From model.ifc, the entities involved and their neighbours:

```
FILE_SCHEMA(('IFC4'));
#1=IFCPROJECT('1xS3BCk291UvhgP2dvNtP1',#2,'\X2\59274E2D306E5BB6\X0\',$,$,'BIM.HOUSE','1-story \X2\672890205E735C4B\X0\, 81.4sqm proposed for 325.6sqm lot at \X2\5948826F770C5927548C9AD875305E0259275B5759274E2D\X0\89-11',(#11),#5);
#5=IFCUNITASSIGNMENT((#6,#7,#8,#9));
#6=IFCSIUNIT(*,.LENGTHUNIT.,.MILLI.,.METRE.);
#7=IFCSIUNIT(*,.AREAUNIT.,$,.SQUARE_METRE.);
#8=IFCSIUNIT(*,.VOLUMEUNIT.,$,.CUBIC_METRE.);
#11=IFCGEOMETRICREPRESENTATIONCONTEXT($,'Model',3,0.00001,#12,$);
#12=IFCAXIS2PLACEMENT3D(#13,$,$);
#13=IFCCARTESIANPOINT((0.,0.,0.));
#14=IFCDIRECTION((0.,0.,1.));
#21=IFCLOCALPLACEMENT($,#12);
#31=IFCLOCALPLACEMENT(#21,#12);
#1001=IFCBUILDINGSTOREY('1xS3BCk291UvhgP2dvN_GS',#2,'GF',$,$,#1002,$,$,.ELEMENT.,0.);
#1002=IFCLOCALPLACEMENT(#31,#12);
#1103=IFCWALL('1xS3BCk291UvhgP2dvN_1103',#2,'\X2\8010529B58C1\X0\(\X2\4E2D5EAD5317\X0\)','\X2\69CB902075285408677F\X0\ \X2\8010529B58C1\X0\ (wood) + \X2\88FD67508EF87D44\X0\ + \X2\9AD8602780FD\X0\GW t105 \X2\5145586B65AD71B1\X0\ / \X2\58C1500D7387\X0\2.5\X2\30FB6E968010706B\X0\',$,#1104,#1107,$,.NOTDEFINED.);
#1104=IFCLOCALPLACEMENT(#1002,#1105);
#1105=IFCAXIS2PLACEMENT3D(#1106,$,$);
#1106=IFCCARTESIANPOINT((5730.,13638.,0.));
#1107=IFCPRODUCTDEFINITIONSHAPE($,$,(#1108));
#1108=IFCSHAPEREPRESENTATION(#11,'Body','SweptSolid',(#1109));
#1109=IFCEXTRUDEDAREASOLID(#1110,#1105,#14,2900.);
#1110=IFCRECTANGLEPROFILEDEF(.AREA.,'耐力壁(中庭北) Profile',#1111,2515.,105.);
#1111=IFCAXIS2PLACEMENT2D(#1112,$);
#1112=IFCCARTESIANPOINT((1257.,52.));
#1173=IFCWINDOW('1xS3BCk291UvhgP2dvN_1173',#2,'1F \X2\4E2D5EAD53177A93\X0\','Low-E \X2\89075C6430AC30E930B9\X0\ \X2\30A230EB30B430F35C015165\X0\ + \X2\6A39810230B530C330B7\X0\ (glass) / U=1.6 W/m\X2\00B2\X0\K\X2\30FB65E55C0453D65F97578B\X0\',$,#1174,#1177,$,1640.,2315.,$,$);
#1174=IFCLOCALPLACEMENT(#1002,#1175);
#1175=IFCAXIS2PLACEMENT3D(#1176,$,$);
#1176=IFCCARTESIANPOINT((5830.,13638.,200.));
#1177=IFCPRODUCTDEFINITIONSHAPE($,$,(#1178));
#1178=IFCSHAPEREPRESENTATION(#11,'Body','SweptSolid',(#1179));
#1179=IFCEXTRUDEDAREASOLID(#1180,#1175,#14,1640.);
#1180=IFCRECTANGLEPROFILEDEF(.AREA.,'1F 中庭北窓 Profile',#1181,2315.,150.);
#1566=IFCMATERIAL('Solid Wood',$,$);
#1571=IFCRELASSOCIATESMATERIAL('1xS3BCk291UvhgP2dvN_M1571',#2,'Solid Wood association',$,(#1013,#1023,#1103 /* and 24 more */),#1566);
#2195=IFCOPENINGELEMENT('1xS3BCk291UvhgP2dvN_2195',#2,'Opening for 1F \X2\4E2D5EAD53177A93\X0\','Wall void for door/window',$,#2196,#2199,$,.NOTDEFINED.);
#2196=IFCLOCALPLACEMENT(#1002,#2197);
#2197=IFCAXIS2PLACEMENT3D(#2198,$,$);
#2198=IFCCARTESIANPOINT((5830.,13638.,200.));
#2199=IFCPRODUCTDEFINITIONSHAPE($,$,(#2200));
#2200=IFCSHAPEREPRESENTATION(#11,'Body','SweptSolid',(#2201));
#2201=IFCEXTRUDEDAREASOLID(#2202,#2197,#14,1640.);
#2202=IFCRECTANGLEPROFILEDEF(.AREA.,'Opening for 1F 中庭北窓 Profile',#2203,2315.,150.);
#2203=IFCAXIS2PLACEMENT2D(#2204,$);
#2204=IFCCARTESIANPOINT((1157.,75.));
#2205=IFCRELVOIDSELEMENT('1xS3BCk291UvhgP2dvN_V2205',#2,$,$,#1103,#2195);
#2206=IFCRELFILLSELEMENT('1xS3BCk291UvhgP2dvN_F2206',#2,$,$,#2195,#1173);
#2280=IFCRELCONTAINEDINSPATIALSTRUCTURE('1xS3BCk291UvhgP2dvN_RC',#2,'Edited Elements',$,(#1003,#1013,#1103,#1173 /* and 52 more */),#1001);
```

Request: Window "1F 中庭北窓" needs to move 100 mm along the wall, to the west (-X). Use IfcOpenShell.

```python
import ifcopenshell
import ifcopenshell.api.geometry
import ifcopenshell.util.placement

model = ifcopenshell.open("model.ifc")

window = model.by_guid("1xS3BCk291UvhgP2dvN_1173")
opening = window.FillsVoids[0].RelatingOpeningElement
wall = opening.VoidsElements[0].RelatingBuildingElement

wall_matrix = ifcopenshell.util.placement.get_local_placement(wall.ObjectPlacement)
shift = wall_matrix[:3, 0] * -100.0
before = ifcopenshell.util.placement.get_local_placement(window.ObjectPlacement)[:3, 3].copy()

# The window is not placed relative to its opening, so move both.
for product in (opening, window):
    matrix = ifcopenshell.util.placement.get_local_placement(product.ObjectPlacement)
    matrix[:3, 3] += shift
    ifcopenshell.api.geometry.edit_object_placement(model, product=product, matrix=matrix, is_si=False)

after = ifcopenshell.util.placement.get_local_placement(window.ObjectPlacement)[:3, 3]
print("window moved by", (after - before).round(3) + 0.0)

model.write("model_v2.ifc")
```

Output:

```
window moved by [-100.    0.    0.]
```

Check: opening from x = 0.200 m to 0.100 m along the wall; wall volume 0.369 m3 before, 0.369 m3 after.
